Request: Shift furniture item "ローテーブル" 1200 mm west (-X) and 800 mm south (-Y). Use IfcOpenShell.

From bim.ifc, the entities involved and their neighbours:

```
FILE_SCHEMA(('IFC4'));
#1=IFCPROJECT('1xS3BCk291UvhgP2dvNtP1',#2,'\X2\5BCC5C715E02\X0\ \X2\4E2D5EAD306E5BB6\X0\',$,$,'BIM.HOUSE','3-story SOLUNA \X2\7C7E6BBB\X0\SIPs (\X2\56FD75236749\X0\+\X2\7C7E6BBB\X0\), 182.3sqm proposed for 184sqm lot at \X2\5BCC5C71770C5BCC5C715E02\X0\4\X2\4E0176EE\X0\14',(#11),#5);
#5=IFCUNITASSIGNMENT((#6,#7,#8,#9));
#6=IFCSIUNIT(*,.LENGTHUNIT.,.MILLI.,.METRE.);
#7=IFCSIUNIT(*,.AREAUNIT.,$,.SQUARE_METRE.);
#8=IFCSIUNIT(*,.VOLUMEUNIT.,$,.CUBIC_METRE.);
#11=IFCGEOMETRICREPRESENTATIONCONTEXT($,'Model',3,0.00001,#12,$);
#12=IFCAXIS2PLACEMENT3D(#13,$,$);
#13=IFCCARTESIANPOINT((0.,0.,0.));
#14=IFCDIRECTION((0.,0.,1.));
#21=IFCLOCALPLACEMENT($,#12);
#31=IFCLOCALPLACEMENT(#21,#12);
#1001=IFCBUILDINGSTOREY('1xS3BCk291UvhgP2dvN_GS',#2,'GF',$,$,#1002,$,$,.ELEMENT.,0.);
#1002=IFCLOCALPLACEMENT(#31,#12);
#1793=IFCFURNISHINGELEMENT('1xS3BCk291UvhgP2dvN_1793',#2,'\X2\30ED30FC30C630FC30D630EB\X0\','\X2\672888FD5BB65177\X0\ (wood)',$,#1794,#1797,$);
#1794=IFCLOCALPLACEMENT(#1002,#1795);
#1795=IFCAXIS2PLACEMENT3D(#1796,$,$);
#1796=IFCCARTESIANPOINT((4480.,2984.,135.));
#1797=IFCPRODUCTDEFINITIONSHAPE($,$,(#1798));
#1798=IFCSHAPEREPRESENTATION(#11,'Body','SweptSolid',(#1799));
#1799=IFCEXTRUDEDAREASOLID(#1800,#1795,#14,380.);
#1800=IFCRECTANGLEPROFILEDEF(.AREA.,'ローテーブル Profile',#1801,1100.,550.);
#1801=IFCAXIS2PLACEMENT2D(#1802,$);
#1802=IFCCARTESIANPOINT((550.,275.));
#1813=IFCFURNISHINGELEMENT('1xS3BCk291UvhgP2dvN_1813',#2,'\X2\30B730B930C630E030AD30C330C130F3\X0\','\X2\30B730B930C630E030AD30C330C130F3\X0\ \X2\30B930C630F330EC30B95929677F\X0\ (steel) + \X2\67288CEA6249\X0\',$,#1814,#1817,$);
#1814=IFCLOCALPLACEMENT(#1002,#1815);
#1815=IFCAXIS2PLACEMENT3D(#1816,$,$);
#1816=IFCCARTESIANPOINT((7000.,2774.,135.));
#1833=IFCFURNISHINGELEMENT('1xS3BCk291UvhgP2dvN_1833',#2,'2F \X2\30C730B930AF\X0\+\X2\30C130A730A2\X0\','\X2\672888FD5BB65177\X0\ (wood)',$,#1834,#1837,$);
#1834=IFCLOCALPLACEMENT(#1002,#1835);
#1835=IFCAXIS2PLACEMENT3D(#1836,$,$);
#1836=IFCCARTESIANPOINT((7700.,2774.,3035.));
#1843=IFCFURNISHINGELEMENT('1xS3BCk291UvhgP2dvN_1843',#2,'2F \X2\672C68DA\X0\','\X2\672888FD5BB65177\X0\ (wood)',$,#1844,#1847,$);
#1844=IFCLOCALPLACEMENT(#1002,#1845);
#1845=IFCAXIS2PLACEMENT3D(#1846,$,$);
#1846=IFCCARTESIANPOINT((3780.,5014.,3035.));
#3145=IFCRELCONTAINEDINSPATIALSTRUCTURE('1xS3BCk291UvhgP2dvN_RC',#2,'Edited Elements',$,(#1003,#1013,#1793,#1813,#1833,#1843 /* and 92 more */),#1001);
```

```python
import ifcopenshell
import ifcopenshell.api.geometry
import ifcopenshell.util.placement

model = ifcopenshell.open("bim.ifc")

item = model.by_guid("1xS3BCk291UvhgP2dvN_1793")
matrix = ifcopenshell.util.placement.get_local_placement(item.ObjectPlacement)
matrix[0, 3] -= 1200.0
matrix[1, 3] -= 800.0
ifcopenshell.api.geometry.edit_object_placement(model, product=item, matrix=matrix, is_si=False)

print(ifcopenshell.util.placement.get_local_placement(item.ObjectPlacement).round(3) + 0.0)

model.write("bim-out.ifc")
```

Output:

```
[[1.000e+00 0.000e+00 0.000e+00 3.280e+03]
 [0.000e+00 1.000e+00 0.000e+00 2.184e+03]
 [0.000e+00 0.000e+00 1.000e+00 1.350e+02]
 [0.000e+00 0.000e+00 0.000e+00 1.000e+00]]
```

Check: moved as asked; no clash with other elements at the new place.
